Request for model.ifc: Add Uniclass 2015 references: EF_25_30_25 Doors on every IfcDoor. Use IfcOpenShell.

First a look at what the model holds.

```python
import ifcopenshell

model = ifcopenshell.open("model.ifc")
print(model.schema)
print("classifications:", [c.Name for c in model.by_type("IfcClassification")])
for ifc_class in ("IfcDoor", "IfcRoof", "IfcStair", "IfcWall", "IfcWindow"):
    print(ifc_class, len(model.by_type(ifc_class)))
```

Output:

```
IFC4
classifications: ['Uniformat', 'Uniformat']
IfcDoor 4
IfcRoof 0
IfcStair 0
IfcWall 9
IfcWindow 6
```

```python
import ifcopenshell
import ifcopenshell.api.classification

model = ifcopenshell.open("model.ifc")

system = ifcopenshell.api.classification.add_classification(model, classification="Uniclass 2015")

codes = {
    "IfcDoor": ("EF_25_30_25", "Doors"),
}
for ifc_class, (code, name) in codes.items():
    products = model.by_type(ifc_class)
    ifcopenshell.api.classification.add_reference(
        model, products=products, classification=system, identification=code, name=name
    )
    print(code, len(products))

model.write("model-out.ifc")
```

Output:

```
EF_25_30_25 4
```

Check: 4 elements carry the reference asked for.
